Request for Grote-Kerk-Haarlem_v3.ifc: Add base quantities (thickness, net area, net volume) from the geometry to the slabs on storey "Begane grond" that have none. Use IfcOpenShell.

First a look at what the model holds.

```python
import ifcopenshell
import ifcopenshell.util.element
import ifcopenshell.util.unit

model = ifcopenshell.open("Grote-Kerk-Haarlem_v3.ifc")
print(model.schema)
for unit_type in ("LENGTHUNIT", "AREAUNIT", "VOLUMEUNIT"):
    print(unit_type, ifcopenshell.util.unit.calculate_unit_scale(model, unit_type))
storey = next(s for s in model.by_type("IfcBuildingStorey") if s.Name == "Begane grond")
slabs = [e for e in ifcopenshell.util.element.get_decomposition(storey) if e.is_a("IfcSlab")]
for e in sorted(slabs, key=lambda e: e.id()):
    print(e.id(), e.is_a(), e.Name, list(ifcopenshell.util.element.get_psets(e, qtos_only=True)), sep=" | ")
```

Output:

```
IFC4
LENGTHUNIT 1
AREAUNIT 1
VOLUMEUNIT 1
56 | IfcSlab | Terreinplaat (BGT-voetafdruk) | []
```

```python
import ifcopenshell
import ifcopenshell.api.pset
import ifcopenshell.geom
import ifcopenshell.util.element
import ifcopenshell.util.shape
import ifcopenshell.util.unit

model = ifcopenshell.open("Grote-Kerk-Haarlem_v3.ifc")
unit_scale = ifcopenshell.util.unit.calculate_unit_scale(model)
area_scale = ifcopenshell.util.unit.calculate_unit_scale(model, "AREAUNIT")
volume_scale = ifcopenshell.util.unit.calculate_unit_scale(model, "VOLUMEUNIT")
settings = ifcopenshell.geom.settings()

storey = next(s for s in model.by_type("IfcBuildingStorey") if s.Name == "Begane grond")
slabs = [e for e in ifcopenshell.util.element.get_decomposition(storey) if e.is_a("IfcSlab")]

for e in sorted(slabs, key=lambda e: e.id()):
    if ifcopenshell.util.element.get_psets(e, qtos_only=True, should_inherit=False):
        continue
    # Geometry comes back in metres, in the element's own axes.
    shape = ifcopenshell.geom.create_shape(settings, e)
    values = {
        "Width": ifcopenshell.util.shape.get_z(shape.geometry) / unit_scale,
        "NetArea": ifcopenshell.util.shape.get_footprint_area(shape.geometry) / area_scale,
        "NetVolume": ifcopenshell.util.shape.get_volume(shape.geometry) / volume_scale,
    }
    qto = ifcopenshell.api.pset.add_qto(model, product=e, name="Qto_SlabBaseQuantities")
    ifcopenshell.api.pset.edit_qto(model, qto=qto, properties=values)
    print(e.id(), {k: round(v, 3) for k, v in values.items()})

model.write("Grote-Kerk-Haarlem_v3_updated.ifc")
```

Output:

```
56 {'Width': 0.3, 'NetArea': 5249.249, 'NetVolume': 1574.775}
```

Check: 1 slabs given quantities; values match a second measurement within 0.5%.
